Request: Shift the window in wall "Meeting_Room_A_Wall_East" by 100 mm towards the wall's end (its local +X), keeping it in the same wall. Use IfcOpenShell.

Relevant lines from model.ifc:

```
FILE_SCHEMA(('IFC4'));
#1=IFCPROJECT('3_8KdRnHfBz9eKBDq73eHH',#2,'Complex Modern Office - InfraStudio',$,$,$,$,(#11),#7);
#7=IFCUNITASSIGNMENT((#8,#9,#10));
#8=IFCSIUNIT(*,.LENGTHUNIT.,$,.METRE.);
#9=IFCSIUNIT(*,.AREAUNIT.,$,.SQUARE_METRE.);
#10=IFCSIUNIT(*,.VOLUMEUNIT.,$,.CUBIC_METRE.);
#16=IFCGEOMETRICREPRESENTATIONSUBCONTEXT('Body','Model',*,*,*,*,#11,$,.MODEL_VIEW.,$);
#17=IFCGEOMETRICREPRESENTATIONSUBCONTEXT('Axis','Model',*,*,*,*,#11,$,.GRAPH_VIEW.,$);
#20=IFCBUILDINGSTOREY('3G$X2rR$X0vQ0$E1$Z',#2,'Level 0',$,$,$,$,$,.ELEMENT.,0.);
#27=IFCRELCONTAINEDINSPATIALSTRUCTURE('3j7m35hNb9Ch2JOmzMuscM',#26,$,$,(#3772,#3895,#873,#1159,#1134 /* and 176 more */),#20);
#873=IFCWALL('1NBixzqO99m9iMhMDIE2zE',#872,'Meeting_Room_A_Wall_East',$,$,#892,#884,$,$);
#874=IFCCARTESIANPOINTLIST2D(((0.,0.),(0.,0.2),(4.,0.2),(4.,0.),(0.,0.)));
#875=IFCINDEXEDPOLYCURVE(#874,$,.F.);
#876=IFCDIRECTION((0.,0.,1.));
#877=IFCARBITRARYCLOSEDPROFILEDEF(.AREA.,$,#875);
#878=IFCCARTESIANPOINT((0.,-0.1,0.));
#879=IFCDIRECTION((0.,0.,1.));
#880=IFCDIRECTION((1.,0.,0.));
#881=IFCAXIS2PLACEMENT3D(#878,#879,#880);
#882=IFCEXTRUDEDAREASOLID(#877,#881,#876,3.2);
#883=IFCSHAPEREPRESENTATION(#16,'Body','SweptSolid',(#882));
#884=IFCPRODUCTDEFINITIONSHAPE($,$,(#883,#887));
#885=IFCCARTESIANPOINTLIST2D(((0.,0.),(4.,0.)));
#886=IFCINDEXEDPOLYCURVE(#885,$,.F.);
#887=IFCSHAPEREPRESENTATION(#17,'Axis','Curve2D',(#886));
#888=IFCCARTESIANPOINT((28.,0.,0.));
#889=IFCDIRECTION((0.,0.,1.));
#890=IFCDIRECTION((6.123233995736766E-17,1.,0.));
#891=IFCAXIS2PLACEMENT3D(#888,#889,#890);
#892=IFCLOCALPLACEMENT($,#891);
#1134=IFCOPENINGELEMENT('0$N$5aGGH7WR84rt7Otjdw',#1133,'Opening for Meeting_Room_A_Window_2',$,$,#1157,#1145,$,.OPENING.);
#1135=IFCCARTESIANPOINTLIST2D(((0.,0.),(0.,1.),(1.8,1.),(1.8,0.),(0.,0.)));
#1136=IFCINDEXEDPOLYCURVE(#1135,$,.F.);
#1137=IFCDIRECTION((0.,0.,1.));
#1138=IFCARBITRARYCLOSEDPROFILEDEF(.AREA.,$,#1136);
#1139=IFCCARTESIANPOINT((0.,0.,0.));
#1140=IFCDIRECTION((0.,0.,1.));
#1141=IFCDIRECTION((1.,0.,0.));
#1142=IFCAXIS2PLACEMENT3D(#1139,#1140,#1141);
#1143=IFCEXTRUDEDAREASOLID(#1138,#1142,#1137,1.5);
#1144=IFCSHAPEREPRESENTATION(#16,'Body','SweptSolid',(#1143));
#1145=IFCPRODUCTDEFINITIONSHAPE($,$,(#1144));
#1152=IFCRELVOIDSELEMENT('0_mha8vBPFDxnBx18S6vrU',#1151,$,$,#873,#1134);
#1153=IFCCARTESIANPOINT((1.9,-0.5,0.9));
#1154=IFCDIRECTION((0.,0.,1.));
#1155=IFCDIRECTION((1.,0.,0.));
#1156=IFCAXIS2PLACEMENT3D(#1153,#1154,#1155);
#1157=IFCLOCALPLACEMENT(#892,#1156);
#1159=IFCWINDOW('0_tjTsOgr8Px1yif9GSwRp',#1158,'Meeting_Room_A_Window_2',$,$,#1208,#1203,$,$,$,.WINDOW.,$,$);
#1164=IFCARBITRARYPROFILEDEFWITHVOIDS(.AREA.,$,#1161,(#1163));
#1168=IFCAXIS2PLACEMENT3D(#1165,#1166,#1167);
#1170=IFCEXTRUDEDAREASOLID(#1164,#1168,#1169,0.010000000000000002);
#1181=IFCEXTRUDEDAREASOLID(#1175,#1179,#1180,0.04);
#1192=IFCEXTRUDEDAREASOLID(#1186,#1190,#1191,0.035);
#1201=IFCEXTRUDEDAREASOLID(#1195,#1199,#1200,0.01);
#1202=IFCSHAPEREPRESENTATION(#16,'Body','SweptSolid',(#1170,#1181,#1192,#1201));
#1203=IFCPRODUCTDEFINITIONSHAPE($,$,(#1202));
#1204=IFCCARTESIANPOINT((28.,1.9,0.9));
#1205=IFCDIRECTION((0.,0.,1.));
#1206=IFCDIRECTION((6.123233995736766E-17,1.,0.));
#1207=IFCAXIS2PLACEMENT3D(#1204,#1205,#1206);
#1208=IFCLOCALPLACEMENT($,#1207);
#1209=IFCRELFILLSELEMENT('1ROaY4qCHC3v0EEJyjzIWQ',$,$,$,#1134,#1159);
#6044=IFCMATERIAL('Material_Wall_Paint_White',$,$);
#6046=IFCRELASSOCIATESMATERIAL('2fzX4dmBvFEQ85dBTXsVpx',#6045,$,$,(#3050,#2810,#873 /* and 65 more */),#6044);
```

```python
import ifcopenshell
import ifcopenshell.api.geometry
import ifcopenshell.util.placement

model = ifcopenshell.open("model.ifc")

window = model.by_id(1159)
opening = window.FillsVoids[0].RelatingOpeningElement
wall = opening.VoidsElements[0].RelatingBuildingElement

wall_matrix = ifcopenshell.util.placement.get_local_placement(wall.ObjectPlacement)
shift = wall_matrix[:3, 0] * 0.1
before = ifcopenshell.util.placement.get_local_placement(window.ObjectPlacement)[:3, 3].copy()

# The window is not placed relative to its opening, so move both.
for product in (opening, window):
    matrix = ifcopenshell.util.placement.get_local_placement(product.ObjectPlacement)
    matrix[:3, 3] += shift
    ifcopenshell.api.geometry.edit_object_placement(model, product=product, matrix=matrix, is_si=False)

after = ifcopenshell.util.placement.get_local_placement(window.ObjectPlacement)[:3, 3]
print("window moved by", (after - before).round(3) + 0.0)

model.write("model_v2.ifc")
```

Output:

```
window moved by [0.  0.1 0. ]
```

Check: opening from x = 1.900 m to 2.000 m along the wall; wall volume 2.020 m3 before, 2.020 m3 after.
